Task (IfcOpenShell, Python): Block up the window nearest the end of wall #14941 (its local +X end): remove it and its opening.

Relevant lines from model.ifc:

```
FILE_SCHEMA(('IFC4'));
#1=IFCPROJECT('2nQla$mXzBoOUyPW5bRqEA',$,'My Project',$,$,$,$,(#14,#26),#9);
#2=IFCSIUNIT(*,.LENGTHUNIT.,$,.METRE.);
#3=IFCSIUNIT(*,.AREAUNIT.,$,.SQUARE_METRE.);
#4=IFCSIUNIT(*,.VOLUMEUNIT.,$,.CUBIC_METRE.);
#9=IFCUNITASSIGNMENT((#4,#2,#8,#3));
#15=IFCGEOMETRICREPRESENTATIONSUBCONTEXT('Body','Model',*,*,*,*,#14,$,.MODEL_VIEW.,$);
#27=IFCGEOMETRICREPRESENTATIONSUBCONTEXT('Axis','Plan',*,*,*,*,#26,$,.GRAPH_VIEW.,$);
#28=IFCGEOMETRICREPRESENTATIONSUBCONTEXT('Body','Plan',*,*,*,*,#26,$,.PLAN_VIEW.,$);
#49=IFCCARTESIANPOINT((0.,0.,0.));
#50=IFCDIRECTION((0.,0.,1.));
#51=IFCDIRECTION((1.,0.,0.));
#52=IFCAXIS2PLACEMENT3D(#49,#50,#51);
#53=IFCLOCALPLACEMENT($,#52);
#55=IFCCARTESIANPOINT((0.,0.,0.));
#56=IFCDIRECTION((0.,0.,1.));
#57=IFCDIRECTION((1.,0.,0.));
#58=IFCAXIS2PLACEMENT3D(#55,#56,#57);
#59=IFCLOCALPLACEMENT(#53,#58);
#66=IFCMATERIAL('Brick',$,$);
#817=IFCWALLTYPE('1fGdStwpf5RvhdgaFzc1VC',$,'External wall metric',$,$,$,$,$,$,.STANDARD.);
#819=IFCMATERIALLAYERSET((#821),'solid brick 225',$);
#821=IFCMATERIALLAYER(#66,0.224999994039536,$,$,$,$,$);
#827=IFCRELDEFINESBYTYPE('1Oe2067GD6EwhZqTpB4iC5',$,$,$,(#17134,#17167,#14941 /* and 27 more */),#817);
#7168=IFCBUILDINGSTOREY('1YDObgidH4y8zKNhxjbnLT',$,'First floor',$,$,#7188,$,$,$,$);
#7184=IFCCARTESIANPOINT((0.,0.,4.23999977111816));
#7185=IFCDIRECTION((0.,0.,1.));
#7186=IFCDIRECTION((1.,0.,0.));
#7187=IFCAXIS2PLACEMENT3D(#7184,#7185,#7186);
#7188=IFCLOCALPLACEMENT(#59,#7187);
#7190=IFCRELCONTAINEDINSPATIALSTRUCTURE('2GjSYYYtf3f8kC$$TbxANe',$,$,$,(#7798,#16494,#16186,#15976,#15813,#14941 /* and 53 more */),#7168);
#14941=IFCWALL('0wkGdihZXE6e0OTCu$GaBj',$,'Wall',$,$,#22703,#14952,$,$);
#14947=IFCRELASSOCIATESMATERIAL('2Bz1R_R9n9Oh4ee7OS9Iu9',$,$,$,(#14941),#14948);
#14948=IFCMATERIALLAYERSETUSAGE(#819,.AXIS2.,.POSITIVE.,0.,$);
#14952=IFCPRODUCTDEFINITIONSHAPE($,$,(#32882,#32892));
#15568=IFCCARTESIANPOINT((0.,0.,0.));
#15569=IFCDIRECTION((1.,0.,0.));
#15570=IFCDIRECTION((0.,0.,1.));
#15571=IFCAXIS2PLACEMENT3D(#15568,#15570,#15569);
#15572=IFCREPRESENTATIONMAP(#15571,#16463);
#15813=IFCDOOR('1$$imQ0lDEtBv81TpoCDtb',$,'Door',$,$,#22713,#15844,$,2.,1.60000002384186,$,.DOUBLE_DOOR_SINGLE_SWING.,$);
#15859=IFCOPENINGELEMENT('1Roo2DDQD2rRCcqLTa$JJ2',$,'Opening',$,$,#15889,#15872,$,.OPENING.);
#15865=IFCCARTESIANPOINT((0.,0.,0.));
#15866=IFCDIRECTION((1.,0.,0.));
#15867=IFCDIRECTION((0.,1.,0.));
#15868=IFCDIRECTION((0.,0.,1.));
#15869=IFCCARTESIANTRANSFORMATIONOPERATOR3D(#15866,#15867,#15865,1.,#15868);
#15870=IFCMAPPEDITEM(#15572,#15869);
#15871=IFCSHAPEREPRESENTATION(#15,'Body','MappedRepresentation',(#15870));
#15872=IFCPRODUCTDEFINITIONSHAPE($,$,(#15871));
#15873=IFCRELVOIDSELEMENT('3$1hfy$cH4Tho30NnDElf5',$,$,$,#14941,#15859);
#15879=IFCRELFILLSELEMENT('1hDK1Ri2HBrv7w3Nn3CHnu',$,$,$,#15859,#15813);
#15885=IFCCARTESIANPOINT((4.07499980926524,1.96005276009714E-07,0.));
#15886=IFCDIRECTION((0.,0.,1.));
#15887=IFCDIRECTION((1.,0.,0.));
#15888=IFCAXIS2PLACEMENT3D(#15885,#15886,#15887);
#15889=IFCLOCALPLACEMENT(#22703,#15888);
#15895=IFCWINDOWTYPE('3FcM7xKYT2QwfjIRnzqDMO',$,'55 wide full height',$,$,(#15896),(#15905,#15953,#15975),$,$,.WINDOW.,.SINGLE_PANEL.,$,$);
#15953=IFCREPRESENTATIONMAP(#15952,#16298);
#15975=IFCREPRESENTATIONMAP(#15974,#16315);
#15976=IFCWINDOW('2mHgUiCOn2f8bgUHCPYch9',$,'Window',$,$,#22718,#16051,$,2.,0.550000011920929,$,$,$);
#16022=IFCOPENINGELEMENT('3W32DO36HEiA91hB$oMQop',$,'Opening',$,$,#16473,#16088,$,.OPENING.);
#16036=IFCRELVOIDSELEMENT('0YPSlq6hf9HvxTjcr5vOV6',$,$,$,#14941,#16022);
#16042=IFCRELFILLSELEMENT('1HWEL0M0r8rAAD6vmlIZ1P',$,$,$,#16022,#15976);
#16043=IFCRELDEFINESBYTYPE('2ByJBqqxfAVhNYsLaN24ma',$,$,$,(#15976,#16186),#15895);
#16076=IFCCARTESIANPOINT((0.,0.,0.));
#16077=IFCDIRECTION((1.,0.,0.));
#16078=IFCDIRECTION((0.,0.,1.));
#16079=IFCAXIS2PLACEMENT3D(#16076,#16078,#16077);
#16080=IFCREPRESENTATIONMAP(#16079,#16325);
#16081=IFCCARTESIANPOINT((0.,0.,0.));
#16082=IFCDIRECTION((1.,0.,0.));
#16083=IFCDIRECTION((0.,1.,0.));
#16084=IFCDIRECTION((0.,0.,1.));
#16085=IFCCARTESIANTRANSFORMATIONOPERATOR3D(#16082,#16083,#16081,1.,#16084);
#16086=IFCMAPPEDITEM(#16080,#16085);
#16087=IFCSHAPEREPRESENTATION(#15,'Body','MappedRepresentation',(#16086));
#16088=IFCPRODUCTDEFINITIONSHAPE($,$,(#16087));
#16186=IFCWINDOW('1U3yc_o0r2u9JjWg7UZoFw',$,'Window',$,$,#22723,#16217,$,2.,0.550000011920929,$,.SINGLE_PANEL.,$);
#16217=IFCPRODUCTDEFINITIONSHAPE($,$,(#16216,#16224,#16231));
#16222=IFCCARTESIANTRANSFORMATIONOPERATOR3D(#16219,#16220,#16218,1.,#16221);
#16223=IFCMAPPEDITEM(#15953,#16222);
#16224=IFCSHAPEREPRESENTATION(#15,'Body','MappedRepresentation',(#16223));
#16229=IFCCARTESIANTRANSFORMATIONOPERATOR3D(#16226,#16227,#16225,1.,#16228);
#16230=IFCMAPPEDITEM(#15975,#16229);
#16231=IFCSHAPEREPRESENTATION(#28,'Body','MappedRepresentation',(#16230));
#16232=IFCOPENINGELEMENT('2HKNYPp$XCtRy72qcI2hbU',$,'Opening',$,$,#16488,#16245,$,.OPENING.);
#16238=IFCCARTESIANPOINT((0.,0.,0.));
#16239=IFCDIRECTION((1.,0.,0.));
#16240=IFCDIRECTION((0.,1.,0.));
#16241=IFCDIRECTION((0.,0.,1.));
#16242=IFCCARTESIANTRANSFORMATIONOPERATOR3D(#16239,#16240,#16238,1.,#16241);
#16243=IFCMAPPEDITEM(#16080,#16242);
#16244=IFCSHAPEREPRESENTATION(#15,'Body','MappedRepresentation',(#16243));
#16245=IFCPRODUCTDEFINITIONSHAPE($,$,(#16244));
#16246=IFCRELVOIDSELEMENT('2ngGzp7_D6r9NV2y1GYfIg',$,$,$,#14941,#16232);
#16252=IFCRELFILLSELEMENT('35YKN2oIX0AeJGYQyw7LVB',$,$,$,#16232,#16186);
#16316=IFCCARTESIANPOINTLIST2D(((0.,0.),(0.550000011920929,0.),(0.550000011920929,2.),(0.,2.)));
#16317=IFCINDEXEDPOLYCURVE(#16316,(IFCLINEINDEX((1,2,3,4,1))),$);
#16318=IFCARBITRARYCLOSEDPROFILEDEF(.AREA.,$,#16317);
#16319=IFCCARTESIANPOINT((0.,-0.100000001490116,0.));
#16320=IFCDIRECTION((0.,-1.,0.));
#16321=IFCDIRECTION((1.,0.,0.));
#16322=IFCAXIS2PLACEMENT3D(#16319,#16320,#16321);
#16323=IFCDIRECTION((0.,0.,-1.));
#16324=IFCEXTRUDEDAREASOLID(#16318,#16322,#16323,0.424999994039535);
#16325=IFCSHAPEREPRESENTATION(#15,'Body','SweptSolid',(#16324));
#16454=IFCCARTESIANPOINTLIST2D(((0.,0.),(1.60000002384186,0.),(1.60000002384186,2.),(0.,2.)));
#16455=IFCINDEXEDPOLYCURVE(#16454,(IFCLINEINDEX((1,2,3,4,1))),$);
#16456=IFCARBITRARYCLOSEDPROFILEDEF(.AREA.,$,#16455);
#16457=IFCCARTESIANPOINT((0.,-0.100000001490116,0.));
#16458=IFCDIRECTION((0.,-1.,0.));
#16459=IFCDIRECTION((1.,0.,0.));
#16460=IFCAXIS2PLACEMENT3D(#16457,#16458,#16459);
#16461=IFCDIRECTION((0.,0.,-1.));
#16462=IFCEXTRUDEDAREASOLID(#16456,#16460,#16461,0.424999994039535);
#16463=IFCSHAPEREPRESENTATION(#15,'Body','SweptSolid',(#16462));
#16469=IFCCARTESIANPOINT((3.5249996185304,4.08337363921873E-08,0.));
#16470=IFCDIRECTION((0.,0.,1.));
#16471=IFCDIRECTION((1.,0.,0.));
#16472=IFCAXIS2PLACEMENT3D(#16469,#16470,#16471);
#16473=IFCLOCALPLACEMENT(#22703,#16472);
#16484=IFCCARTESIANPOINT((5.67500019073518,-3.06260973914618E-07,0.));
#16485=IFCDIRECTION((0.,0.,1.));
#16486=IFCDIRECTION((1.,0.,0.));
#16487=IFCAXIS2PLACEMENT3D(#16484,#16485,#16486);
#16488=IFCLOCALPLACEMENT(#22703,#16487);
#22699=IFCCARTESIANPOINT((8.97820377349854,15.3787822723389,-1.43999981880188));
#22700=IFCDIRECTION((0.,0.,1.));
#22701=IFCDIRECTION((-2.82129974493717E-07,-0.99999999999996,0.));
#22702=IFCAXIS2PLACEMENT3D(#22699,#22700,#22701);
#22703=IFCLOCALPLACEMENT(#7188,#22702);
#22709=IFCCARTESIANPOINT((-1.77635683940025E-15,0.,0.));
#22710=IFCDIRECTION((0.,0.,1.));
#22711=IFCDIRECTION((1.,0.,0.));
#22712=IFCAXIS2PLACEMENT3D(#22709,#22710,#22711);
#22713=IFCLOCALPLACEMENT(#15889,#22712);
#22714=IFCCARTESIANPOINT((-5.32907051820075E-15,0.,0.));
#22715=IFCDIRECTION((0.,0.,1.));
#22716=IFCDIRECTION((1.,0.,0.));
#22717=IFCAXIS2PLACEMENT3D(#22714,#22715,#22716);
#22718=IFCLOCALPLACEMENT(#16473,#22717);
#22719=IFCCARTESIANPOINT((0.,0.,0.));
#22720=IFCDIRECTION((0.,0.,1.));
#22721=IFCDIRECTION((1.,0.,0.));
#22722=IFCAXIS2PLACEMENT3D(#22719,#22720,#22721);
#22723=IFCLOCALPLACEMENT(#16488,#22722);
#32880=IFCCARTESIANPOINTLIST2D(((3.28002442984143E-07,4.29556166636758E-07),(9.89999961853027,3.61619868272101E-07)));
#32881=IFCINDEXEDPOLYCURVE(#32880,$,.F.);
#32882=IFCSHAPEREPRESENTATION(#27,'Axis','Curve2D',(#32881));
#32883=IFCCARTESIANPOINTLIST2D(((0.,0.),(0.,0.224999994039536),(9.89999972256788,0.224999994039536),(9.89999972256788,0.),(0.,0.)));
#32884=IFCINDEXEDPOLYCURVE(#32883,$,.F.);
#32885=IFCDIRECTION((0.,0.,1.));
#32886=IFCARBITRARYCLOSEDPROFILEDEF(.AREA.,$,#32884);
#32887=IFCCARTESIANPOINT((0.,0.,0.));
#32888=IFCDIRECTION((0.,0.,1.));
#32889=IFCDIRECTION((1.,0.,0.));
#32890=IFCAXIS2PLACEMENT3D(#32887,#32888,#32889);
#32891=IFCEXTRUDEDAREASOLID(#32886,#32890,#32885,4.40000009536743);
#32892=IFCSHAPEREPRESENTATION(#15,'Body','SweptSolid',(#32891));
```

```python
import ifcopenshell
import ifcopenshell.api.feature
import ifcopenshell.api.root
import ifcopenshell.geom
import ifcopenshell.util.shape

model = ifcopenshell.open("model.ifc")
settings = ifcopenshell.geom.settings()


def volume(element):
    """Net volume in cubic metres, openings subtracted."""
    shape = ifcopenshell.geom.create_shape(settings, element)
    return ifcopenshell.util.shape.get_volume(shape.geometry)


window = model.by_guid("1U3yc_o0r2u9JjWg7UZoFw")
opening = window.FillsVoids[0].RelatingOpeningElement
wall = opening.VoidsElements[0].RelatingBuildingElement
before = volume(wall)

ifcopenshell.api.root.remove_product(model, product=window)
ifcopenshell.api.feature.remove_feature(model, feature=opening)

after = volume(wall)

print(f"wall volume {before:.3f} -> {after:.3f} m3")

model.write("model_updated.ifc")
```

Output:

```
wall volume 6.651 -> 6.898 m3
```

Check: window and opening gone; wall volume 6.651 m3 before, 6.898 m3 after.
